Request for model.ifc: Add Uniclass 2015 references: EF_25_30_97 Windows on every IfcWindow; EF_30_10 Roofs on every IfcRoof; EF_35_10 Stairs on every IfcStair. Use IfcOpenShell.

First a look at what the model holds.

```python
import ifcopenshell

model = ifcopenshell.open("model.ifc")
print(model.schema)
print("classifications:", [c.Name for c in model.by_type("IfcClassification")])
for ifc_class in ("IfcDoor", "IfcRoof", "IfcStair", "IfcWall", "IfcWindow"):
    print(ifc_class, len(model.by_type(ifc_class)))
```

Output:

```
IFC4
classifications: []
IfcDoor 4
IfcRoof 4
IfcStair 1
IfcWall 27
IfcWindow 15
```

```python
import ifcopenshell
import ifcopenshell.api.classification

model = ifcopenshell.open("model.ifc")

system = ifcopenshell.api.classification.add_classification(model, classification="Uniclass 2015")

codes = {
    "IfcWindow": ("EF_25_30_97", "Windows"),
    "IfcRoof": ("EF_30_10", "Roofs"),
    "IfcStair": ("EF_35_10", "Stairs"),
}
for ifc_class, (code, name) in codes.items():
    products = model.by_type(ifc_class)
    ifcopenshell.api.classification.add_reference(
        model, products=products, classification=system, identification=code, name=name
    )
    print(code, len(products))

model.write("model_updated.ifc")
```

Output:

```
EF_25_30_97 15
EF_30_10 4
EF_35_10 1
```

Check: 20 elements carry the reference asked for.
